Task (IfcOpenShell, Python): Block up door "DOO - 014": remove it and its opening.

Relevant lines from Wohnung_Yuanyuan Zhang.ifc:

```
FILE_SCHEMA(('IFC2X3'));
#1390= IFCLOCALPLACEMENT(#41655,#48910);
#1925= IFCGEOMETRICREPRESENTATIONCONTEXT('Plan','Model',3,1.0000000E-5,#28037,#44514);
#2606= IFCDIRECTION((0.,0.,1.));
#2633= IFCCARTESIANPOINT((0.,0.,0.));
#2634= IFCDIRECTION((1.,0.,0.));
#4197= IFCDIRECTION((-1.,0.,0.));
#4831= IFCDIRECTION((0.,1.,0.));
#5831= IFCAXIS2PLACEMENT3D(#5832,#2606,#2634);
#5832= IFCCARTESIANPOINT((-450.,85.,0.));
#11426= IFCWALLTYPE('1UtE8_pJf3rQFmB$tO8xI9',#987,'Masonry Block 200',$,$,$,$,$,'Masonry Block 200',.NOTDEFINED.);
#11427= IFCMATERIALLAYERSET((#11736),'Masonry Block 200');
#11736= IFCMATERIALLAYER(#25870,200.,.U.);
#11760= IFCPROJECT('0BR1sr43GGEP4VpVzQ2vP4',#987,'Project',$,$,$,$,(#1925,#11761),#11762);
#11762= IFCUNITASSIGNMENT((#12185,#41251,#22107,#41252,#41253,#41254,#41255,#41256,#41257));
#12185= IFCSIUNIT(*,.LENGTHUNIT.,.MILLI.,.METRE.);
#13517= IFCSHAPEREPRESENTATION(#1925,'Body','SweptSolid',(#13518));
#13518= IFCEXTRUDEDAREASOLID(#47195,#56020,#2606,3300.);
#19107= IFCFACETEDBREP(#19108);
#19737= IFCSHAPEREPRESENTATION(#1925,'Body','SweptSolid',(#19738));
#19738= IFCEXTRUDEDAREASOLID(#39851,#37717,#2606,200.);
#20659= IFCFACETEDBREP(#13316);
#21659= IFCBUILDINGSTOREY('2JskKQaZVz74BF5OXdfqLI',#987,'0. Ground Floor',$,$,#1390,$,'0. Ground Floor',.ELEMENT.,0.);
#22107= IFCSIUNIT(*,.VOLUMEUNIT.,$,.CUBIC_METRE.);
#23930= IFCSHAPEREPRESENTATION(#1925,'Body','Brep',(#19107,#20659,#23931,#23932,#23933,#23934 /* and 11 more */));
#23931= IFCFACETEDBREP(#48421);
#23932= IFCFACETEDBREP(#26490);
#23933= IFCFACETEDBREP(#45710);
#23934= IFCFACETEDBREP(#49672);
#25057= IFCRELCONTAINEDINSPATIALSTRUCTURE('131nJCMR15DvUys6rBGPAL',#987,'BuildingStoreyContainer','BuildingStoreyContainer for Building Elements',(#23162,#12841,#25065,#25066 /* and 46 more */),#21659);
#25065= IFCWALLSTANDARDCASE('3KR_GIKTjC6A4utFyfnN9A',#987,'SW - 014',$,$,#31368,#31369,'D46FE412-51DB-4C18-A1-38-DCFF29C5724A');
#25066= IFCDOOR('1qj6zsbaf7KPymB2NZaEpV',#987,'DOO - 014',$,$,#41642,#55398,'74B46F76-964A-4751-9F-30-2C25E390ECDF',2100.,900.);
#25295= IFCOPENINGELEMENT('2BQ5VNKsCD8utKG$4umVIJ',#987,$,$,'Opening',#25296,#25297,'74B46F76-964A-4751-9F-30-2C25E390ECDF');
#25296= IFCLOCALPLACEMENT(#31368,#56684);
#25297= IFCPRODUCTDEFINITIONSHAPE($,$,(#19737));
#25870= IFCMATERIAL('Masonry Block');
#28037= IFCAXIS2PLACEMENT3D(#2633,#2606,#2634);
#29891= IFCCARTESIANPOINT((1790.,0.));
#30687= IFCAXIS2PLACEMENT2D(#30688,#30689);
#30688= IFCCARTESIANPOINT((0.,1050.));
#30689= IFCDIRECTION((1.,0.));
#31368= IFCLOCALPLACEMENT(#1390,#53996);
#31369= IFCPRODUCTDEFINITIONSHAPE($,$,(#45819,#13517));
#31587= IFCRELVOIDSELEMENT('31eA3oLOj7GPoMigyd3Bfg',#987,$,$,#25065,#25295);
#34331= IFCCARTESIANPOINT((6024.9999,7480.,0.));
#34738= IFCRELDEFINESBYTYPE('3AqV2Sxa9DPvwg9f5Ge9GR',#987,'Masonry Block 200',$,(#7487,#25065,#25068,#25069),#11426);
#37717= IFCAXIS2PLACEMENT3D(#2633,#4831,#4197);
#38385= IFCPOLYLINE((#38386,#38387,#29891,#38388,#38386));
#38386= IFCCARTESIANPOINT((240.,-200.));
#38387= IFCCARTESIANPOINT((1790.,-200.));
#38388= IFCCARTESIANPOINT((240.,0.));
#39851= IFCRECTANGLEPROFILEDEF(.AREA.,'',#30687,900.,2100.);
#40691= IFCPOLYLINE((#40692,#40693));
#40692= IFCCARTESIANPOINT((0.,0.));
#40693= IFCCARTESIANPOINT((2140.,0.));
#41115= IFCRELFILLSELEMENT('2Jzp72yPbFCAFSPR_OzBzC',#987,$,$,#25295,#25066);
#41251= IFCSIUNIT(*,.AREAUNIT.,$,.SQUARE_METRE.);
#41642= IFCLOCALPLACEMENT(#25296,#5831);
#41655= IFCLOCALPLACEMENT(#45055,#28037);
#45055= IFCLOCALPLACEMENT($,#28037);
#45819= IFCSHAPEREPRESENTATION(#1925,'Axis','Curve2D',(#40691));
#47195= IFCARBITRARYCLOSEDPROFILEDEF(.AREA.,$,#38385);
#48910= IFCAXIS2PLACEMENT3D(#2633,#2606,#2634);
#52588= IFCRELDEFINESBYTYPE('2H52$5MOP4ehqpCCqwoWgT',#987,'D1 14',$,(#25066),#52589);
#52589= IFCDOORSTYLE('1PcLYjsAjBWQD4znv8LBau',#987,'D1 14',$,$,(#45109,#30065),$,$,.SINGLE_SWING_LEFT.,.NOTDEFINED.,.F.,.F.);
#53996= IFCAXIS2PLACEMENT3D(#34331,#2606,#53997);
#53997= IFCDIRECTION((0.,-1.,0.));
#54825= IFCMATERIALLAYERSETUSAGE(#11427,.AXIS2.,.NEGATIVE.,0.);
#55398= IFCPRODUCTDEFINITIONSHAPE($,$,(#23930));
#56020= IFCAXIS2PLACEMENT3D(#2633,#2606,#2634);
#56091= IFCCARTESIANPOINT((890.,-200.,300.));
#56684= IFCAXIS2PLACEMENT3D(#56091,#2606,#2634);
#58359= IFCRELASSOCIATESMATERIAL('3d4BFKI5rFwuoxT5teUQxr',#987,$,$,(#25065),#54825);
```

```python
import ifcopenshell
import ifcopenshell.api.feature
import ifcopenshell.api.root
import ifcopenshell.geom
import ifcopenshell.util.shape

model = ifcopenshell.open("Wohnung_Yuanyuan Zhang.ifc")
settings = ifcopenshell.geom.settings()


def volume(element):
    """Net volume in cubic metres, openings subtracted."""
    shape = ifcopenshell.geom.create_shape(settings, element)
    return ifcopenshell.util.shape.get_volume(shape.geometry)


door = model.by_id(25066)
opening = door.FillsVoids[0].RelatingOpeningElement
wall = opening.VoidsElements[0].RelatingBuildingElement
before = volume(wall)

ifcopenshell.api.root.remove_product(model, product=door)
ifcopenshell.api.feature.remove_feature(model, feature=opening)

after = volume(wall)

print(f"wall volume {before:.3f} -> {after:.3f} m3")

model.write("Wohnung_Yuanyuan Zhang_edited.ifc")
```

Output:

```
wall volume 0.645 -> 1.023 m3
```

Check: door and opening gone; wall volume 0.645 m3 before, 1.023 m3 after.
